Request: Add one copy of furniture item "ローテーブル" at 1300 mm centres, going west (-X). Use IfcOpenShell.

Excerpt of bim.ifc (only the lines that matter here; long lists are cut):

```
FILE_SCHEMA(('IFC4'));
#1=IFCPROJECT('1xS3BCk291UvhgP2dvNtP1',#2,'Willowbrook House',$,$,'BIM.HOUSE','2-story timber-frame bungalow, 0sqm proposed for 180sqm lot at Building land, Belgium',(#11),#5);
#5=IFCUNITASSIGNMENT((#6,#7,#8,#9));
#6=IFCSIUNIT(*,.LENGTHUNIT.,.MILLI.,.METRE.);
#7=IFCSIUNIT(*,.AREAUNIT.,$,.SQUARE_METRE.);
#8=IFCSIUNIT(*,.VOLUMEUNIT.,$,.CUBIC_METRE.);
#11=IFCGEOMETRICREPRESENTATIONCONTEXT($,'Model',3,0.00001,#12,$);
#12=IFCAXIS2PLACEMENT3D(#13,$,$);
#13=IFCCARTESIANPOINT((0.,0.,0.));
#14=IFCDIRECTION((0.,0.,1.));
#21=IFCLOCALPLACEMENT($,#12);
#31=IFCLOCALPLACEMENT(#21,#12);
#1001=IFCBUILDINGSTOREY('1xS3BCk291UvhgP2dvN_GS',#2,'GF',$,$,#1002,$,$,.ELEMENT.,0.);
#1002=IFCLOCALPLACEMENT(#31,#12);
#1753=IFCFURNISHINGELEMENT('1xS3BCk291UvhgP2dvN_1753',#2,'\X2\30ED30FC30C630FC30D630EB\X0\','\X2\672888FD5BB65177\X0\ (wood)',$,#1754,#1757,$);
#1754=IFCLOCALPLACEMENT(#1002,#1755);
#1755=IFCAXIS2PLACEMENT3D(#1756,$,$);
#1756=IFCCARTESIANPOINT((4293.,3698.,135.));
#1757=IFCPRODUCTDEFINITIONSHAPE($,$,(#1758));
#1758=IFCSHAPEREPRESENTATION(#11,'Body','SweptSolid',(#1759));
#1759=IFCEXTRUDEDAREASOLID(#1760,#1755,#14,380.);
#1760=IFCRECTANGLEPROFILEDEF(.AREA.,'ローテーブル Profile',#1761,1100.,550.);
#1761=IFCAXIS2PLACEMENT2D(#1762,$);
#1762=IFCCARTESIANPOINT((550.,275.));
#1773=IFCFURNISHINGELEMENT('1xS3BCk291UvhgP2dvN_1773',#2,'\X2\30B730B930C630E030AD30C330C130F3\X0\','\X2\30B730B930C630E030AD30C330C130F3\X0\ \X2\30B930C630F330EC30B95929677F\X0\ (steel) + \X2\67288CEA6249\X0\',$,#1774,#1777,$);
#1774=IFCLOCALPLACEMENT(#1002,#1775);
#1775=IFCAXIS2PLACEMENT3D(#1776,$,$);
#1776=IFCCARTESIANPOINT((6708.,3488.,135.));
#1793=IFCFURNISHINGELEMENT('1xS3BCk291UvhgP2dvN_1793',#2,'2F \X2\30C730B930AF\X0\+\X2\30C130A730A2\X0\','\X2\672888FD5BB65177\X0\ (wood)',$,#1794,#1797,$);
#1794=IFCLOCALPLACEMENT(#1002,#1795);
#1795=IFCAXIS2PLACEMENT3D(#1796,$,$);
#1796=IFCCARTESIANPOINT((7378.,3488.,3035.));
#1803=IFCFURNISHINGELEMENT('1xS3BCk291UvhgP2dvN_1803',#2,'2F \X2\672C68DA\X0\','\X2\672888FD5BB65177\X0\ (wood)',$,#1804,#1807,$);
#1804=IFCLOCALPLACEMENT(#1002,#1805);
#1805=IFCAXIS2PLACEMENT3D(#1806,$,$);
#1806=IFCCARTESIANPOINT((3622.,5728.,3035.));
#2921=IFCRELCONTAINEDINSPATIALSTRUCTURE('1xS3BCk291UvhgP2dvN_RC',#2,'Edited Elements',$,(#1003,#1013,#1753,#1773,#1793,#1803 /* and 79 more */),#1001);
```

```python
import numpy as np
import ifcopenshell
import ifcopenshell.api.geometry
import ifcopenshell.api.root
import ifcopenshell.util.element
import ifcopenshell.util.placement

model = ifcopenshell.open("bim.ifc")


def reuse_history(source, copy):
    """copy_class also copies each property set's owner history, people and application; keep the originals."""
    for rel in copy.IsDefinedBy:
        if rel.is_a("IfcRelDefinesByProperties") and (history := rel.RelatingPropertyDefinition.OwnerHistory):
            rel.RelatingPropertyDefinition.OwnerHistory = source.OwnerHistory
            ifcopenshell.util.element.remove_deep2(model, history)


source = model.by_id(1753)
base = ifcopenshell.util.placement.get_local_placement(source.ObjectPlacement)
step = np.array([-1.0, 0.0, 0.0]) * 1300.0

for i in range(1, 2):
    copy = ifcopenshell.api.root.copy_class(model, product=source)
    copy.Representation = ifcopenshell.util.element.copy_deep(
        model, source.Representation, exclude=["IfcGeometricRepresentationContext", "IfcRepresentationMap"]
    )
    reuse_history(source, copy)
    matrix = base.copy()
    matrix[:3, 3] += i * step
    print("added at", matrix[:3, 3].round(3) + 0.0)
    ifcopenshell.api.geometry.edit_object_placement(model, product=copy, matrix=matrix, is_si=False)

model.write("bim-out.ifc")
```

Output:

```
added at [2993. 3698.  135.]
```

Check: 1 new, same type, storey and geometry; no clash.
